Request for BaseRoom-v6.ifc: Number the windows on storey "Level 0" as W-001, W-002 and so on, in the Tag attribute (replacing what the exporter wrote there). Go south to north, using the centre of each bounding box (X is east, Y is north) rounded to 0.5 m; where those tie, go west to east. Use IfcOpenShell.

First a look at what the model holds.

```python
import ifcopenshell
import ifcopenshell.util.element
import ifcopenshell.util.placement

model = ifcopenshell.open("BaseRoom-v6.ifc")
print(model.schema)
storey = next(s for s in model.by_type("IfcBuildingStorey") if s.Name == "Level 0")
windows = [e for e in ifcopenshell.util.element.get_decomposition(storey) if e.is_a("IfcWindow")]
for e in sorted(windows, key=lambda e: e.id()):
    origin = ifcopenshell.util.placement.get_local_placement(e.ObjectPlacement)[:3, 3]
    print(e.id(), e.Tag, e.Name, origin.round(2) + 0.0, sep=" | ")
```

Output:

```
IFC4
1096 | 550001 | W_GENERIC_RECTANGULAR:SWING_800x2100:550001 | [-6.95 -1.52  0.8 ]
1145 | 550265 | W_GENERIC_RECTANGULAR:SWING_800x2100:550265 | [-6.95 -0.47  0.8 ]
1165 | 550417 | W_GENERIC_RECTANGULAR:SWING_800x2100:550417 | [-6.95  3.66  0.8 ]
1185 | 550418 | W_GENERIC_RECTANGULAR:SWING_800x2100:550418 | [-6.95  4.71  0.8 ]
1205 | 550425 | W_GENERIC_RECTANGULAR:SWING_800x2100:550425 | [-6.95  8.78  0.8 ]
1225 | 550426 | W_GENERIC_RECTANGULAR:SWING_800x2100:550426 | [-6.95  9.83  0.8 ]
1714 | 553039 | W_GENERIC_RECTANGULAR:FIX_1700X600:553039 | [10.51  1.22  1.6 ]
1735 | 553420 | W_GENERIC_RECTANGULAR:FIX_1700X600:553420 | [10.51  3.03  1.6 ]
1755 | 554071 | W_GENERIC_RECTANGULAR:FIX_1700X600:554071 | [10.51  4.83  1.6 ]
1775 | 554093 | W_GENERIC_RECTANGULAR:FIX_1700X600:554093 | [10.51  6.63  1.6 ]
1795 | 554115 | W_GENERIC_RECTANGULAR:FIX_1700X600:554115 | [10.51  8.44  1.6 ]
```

```python
import ifcopenshell
import ifcopenshell.geom
import ifcopenshell.util.element
import ifcopenshell.util.shape

model = ifcopenshell.open("BaseRoom-v6.ifc")
settings = ifcopenshell.geom.settings()
settings.set("use-world-coords", True)


def centre(element):
    shape = ifcopenshell.geom.create_shape(settings, element)
    return ifcopenshell.util.shape.get_bbox_centroid(shape.geometry)


storey = next(s for s in model.by_type("IfcBuildingStorey") if s.Name == "Level 0")
windows = [e for e in ifcopenshell.util.element.get_decomposition(storey) if e.is_a("IfcWindow")]

# Insertion points can sit at a corner or the storey origin, so sort by the geometry (in metres).
centres = {e: centre(e) for e in windows}
windows.sort(key=lambda e: (round(centres[e][1] / 0.5), centres[e][0]))

for i, e in enumerate(windows, start=1):
    number = f"W-0{i:02d}"
    e.Tag = number
    print(e.id(), number)

model.write("BaseRoom-v6_rev.ifc")
```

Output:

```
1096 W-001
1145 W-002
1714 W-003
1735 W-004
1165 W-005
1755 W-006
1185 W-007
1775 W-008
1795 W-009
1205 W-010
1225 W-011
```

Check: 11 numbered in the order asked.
